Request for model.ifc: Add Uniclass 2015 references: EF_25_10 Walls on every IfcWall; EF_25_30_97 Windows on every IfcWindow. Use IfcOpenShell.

First a look at what the model holds.

```python
import ifcopenshell

model = ifcopenshell.open("model.ifc")
print(model.schema)
print("classifications:", [c.Name for c in model.by_type("IfcClassification")])
for ifc_class in ("IfcDoor", "IfcRoof", "IfcStair", "IfcWall", "IfcWindow"):
    print(ifc_class, len(model.by_type(ifc_class)))
```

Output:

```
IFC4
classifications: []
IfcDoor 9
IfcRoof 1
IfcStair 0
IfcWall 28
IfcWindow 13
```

```python
import ifcopenshell
import ifcopenshell.api.classification

model = ifcopenshell.open("model.ifc")

system = ifcopenshell.api.classification.add_classification(model, classification="Uniclass 2015")

codes = {
    "IfcWall": ("EF_25_10", "Walls"),
    "IfcWindow": ("EF_25_30_97", "Windows"),
}
for ifc_class, (code, name) in codes.items():
    products = model.by_type(ifc_class)
    ifcopenshell.api.classification.add_reference(
        model, products=products, classification=system, identification=code, name=name
    )
    print(code, len(products))

model.write("model_v2.ifc")
```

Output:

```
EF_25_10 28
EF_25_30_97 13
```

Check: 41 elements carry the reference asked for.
